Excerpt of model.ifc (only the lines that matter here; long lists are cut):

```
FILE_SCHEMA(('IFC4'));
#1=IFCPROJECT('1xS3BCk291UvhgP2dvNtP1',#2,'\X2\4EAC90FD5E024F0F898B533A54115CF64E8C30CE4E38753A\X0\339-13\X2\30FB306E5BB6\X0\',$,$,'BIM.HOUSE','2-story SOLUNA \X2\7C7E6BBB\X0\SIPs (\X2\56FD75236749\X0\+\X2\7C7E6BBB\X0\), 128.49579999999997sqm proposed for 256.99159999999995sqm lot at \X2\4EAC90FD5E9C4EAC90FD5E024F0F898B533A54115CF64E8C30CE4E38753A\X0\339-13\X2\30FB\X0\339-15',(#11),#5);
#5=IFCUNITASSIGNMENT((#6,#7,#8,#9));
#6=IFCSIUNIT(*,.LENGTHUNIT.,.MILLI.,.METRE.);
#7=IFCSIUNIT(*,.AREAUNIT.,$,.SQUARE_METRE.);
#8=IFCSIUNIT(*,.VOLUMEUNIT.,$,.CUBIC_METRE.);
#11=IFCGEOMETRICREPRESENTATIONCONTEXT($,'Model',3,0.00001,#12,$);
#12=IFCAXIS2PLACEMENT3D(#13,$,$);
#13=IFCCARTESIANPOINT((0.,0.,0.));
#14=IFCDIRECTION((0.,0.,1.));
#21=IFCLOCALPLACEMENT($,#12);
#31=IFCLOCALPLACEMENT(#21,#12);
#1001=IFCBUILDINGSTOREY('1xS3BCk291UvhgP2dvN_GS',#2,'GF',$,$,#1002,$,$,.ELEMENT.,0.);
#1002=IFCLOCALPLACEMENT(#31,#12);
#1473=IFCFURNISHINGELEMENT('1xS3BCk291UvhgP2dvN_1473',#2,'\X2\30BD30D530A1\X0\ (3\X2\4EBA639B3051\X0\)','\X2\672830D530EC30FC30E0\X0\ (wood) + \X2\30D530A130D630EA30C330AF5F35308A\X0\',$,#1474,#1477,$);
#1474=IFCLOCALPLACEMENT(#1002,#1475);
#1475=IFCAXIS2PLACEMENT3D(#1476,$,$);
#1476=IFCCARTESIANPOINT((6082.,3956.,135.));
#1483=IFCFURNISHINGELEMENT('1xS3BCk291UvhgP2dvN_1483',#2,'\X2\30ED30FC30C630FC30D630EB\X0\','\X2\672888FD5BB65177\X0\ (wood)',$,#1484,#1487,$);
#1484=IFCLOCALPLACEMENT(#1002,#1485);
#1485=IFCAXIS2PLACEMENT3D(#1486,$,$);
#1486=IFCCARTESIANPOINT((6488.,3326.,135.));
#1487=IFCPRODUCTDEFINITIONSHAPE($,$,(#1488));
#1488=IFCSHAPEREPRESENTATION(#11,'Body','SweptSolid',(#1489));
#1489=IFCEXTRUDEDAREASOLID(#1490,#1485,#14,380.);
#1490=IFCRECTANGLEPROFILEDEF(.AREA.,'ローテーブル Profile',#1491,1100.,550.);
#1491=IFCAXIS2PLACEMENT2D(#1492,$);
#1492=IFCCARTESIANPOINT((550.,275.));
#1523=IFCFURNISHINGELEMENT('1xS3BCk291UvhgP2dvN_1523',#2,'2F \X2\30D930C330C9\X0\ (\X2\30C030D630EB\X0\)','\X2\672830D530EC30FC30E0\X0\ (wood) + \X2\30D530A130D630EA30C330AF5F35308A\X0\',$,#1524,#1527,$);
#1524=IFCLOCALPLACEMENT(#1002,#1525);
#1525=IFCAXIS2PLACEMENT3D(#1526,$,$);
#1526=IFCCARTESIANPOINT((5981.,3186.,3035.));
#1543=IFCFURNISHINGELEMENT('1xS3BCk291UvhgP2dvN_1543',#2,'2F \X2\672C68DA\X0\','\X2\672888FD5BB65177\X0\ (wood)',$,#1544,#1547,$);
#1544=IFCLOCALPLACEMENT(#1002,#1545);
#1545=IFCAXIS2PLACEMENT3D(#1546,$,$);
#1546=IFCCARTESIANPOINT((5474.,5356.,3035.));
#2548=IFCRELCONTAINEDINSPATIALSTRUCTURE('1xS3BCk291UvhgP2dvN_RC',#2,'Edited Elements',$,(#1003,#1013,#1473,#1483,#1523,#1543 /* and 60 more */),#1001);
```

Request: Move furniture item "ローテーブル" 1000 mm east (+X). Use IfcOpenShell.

```python
import ifcopenshell
import ifcopenshell.api.geometry
import ifcopenshell.util.placement
import ifcopenshell.util.unit

model = ifcopenshell.open("model.ifc")
unit_scale = ifcopenshell.util.unit.calculate_unit_scale(model)

item = model.by_guid("1xS3BCk291UvhgP2dvN_1483")
matrix = ifcopenshell.util.placement.get_local_placement(item.ObjectPlacement)
matrix[0, 3] += 1 / unit_scale
ifcopenshell.api.geometry.edit_object_placement(model, product=item, matrix=matrix, is_si=False)

print(ifcopenshell.util.placement.get_local_placement(item.ObjectPlacement).round(3) + 0.0)

model.write("model_updated.ifc")
```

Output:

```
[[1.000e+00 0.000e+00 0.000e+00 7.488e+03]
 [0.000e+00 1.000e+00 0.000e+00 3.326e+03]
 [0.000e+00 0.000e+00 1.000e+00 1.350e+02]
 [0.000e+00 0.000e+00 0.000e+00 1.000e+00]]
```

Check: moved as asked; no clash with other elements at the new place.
